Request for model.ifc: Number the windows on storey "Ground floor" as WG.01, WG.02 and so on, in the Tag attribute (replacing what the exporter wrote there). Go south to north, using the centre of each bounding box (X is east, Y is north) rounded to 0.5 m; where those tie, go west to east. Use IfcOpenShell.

First a look at what the model holds.

```python
import ifcopenshell
import ifcopenshell.util.element
import ifcopenshell.util.placement

model = ifcopenshell.open("model.ifc")
print(model.schema)
storey = next(s for s in model.by_type("IfcBuildingStorey") if s.Name == "Ground floor")
windows = [e for e in ifcopenshell.util.element.get_decomposition(storey) if e.is_a("IfcWindow")]
for e in sorted(windows, key=lambda e: e.id()):
    origin = ifcopenshell.util.placement.get_local_placement(e.ObjectPlacement)[:3, 3]
    print(e.id(), e.Tag, e.Name, origin.round(2) + 0.0, sep=" | ")
```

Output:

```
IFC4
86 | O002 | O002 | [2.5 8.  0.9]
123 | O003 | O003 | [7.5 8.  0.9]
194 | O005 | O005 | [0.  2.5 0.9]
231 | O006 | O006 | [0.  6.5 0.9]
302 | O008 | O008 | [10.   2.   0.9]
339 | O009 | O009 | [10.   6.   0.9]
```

```python
import ifcopenshell
import ifcopenshell.geom
import ifcopenshell.util.element
import ifcopenshell.util.shape

model = ifcopenshell.open("model.ifc")
settings = ifcopenshell.geom.settings()
settings.set("use-world-coords", True)


def centre(element):
    shape = ifcopenshell.geom.create_shape(settings, element)
    return ifcopenshell.util.shape.get_bbox_centroid(shape.geometry)


storey = next(s for s in model.by_type("IfcBuildingStorey") if s.Name == "Ground floor")
windows = [e for e in ifcopenshell.util.element.get_decomposition(storey) if e.is_a("IfcWindow")]

# Insertion points can sit at a corner or the storey origin, so sort by the geometry (in metres).
centres = {e: centre(e) for e in windows}
windows.sort(key=lambda e: (round(centres[e][1] / 0.5), centres[e][0]))

for i, e in enumerate(windows, start=1):
    number = f"WG.{i:02d}"
    e.Tag = number
    print(e.id(), number)

model.write("model_edited.ifc")
```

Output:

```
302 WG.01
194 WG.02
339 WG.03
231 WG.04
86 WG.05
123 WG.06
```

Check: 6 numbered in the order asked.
